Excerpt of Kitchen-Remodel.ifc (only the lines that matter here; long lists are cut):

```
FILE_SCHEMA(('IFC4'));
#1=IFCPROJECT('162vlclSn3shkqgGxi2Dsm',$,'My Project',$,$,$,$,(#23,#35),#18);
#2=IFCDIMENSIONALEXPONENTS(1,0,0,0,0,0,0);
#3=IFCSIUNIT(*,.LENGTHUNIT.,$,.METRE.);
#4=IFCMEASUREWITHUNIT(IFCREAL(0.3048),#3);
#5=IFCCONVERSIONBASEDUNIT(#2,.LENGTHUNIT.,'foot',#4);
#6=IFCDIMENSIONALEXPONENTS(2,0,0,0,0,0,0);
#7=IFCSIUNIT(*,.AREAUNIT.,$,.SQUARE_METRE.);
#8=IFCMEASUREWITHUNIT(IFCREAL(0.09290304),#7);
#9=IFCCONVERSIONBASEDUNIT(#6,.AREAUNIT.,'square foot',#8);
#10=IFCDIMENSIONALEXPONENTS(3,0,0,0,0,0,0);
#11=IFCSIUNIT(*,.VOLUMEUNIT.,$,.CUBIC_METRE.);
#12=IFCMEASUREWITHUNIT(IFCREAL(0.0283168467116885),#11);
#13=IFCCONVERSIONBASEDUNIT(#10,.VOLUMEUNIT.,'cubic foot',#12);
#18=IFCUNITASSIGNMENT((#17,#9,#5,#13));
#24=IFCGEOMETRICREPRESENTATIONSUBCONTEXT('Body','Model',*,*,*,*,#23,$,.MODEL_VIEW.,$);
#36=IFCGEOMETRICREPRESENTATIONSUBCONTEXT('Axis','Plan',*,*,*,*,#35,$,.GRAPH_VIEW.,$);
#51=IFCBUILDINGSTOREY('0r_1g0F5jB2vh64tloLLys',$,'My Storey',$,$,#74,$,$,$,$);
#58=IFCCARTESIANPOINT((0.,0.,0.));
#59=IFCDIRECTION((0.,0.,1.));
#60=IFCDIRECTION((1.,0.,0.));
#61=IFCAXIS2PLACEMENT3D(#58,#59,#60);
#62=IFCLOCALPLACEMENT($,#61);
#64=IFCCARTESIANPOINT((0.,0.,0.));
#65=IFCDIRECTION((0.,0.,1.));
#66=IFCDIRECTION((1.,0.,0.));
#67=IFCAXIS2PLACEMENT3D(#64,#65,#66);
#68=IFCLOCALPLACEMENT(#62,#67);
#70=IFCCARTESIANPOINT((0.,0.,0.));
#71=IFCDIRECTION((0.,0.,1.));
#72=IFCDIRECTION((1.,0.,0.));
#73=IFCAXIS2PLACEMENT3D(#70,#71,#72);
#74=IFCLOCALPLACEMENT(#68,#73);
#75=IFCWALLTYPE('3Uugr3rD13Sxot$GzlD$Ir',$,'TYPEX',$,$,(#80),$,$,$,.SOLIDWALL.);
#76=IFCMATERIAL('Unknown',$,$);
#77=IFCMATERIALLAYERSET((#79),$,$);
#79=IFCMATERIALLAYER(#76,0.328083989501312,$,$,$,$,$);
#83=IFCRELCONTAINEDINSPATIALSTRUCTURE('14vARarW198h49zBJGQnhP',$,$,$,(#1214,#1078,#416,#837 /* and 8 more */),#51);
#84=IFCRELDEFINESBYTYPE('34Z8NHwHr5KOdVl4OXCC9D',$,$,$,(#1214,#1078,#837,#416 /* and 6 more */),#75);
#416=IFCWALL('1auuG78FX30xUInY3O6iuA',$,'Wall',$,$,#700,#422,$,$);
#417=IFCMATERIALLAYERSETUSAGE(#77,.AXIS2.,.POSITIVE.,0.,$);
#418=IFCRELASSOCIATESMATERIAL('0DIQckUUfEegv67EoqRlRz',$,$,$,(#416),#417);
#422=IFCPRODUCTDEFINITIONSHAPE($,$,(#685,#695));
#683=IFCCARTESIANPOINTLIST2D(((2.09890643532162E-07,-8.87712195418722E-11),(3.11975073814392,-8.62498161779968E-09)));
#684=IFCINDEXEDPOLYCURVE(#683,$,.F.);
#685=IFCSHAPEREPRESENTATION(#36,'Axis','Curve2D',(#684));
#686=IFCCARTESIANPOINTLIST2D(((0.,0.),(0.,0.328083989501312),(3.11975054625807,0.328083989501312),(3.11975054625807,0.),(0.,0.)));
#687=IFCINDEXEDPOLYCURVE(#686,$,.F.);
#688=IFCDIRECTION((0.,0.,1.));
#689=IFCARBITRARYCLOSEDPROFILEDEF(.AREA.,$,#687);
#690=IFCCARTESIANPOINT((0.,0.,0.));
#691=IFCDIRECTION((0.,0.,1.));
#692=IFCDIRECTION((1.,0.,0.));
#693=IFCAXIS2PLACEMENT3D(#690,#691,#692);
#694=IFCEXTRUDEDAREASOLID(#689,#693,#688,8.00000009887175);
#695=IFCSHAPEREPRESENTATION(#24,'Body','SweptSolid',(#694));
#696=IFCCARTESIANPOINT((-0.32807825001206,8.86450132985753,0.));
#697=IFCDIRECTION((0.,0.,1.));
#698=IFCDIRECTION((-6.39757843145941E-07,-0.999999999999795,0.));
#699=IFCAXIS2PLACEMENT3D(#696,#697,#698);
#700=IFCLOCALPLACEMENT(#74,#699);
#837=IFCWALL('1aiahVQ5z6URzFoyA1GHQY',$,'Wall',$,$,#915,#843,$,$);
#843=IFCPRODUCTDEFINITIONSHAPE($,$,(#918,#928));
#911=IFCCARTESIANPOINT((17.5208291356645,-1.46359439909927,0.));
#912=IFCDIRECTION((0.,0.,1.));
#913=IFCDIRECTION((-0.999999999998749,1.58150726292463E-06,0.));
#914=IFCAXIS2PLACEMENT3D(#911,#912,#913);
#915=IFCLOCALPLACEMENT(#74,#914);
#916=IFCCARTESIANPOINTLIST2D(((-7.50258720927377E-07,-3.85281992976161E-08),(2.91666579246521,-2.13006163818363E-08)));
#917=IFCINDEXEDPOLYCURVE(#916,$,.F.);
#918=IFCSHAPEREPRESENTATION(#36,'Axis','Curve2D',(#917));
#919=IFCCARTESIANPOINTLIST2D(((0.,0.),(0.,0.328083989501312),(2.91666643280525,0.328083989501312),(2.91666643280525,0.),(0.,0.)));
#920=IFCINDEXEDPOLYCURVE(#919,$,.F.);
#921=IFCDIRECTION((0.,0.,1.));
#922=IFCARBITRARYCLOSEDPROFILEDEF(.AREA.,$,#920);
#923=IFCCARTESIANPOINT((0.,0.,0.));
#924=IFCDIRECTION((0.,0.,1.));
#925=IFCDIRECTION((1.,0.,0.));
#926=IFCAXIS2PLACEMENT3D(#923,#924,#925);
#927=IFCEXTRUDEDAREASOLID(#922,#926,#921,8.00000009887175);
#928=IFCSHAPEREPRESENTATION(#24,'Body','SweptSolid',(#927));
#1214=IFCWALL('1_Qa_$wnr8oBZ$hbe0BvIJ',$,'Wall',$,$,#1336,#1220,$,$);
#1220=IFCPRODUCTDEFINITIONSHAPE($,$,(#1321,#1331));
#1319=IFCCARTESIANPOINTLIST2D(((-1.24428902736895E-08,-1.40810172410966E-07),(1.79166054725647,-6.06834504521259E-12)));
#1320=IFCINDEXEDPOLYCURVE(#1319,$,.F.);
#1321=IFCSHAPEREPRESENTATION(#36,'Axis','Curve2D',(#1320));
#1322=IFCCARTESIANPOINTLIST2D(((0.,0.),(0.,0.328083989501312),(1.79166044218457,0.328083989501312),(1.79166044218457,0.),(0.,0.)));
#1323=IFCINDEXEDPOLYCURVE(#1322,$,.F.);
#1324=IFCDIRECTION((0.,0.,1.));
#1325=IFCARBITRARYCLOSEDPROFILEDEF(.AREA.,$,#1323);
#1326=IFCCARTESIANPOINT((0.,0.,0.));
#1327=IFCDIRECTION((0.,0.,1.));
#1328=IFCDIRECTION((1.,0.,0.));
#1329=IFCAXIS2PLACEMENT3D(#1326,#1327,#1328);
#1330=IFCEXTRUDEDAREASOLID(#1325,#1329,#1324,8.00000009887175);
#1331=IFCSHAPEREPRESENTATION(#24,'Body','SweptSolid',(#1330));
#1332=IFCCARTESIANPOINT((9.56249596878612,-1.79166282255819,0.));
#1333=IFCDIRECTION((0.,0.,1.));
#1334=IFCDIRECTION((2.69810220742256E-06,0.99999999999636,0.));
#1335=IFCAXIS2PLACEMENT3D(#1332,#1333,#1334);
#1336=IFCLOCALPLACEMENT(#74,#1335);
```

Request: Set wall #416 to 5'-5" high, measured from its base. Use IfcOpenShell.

```python
import ifcopenshell
import ifcopenshell.geom
import ifcopenshell.util.representation
import ifcopenshell.util.shape
import ifcopenshell.util.unit

model = ifcopenshell.open("Kitchen-Remodel.ifc")
unit_scale = ifcopenshell.util.unit.calculate_unit_scale(model)
settings = ifcopenshell.geom.settings()


def volume(element):
    """Net volume in cubic metres, openings subtracted."""
    shape = ifcopenshell.geom.create_shape(settings, element)
    return ifcopenshell.util.shape.get_volume(shape.geometry)


wall = model.by_guid("1auuG78FX30xUInY3O6iuA")
before = volume(wall)

body = ifcopenshell.util.representation.get_representation(wall, "Model", "Body")
solid = body.Items[0]
old_height = solid.Depth
solid.Depth = 65 * 0.0254 / unit_scale
after = volume(wall)

print(f"height {old_height:g} -> {solid.Depth:g}, volume {before:.3f} -> {after:.3f} m3")

model.write("Kitchen-Remodel_edited.ifc")
```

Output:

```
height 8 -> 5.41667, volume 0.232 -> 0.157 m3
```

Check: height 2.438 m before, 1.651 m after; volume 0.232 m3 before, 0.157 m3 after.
